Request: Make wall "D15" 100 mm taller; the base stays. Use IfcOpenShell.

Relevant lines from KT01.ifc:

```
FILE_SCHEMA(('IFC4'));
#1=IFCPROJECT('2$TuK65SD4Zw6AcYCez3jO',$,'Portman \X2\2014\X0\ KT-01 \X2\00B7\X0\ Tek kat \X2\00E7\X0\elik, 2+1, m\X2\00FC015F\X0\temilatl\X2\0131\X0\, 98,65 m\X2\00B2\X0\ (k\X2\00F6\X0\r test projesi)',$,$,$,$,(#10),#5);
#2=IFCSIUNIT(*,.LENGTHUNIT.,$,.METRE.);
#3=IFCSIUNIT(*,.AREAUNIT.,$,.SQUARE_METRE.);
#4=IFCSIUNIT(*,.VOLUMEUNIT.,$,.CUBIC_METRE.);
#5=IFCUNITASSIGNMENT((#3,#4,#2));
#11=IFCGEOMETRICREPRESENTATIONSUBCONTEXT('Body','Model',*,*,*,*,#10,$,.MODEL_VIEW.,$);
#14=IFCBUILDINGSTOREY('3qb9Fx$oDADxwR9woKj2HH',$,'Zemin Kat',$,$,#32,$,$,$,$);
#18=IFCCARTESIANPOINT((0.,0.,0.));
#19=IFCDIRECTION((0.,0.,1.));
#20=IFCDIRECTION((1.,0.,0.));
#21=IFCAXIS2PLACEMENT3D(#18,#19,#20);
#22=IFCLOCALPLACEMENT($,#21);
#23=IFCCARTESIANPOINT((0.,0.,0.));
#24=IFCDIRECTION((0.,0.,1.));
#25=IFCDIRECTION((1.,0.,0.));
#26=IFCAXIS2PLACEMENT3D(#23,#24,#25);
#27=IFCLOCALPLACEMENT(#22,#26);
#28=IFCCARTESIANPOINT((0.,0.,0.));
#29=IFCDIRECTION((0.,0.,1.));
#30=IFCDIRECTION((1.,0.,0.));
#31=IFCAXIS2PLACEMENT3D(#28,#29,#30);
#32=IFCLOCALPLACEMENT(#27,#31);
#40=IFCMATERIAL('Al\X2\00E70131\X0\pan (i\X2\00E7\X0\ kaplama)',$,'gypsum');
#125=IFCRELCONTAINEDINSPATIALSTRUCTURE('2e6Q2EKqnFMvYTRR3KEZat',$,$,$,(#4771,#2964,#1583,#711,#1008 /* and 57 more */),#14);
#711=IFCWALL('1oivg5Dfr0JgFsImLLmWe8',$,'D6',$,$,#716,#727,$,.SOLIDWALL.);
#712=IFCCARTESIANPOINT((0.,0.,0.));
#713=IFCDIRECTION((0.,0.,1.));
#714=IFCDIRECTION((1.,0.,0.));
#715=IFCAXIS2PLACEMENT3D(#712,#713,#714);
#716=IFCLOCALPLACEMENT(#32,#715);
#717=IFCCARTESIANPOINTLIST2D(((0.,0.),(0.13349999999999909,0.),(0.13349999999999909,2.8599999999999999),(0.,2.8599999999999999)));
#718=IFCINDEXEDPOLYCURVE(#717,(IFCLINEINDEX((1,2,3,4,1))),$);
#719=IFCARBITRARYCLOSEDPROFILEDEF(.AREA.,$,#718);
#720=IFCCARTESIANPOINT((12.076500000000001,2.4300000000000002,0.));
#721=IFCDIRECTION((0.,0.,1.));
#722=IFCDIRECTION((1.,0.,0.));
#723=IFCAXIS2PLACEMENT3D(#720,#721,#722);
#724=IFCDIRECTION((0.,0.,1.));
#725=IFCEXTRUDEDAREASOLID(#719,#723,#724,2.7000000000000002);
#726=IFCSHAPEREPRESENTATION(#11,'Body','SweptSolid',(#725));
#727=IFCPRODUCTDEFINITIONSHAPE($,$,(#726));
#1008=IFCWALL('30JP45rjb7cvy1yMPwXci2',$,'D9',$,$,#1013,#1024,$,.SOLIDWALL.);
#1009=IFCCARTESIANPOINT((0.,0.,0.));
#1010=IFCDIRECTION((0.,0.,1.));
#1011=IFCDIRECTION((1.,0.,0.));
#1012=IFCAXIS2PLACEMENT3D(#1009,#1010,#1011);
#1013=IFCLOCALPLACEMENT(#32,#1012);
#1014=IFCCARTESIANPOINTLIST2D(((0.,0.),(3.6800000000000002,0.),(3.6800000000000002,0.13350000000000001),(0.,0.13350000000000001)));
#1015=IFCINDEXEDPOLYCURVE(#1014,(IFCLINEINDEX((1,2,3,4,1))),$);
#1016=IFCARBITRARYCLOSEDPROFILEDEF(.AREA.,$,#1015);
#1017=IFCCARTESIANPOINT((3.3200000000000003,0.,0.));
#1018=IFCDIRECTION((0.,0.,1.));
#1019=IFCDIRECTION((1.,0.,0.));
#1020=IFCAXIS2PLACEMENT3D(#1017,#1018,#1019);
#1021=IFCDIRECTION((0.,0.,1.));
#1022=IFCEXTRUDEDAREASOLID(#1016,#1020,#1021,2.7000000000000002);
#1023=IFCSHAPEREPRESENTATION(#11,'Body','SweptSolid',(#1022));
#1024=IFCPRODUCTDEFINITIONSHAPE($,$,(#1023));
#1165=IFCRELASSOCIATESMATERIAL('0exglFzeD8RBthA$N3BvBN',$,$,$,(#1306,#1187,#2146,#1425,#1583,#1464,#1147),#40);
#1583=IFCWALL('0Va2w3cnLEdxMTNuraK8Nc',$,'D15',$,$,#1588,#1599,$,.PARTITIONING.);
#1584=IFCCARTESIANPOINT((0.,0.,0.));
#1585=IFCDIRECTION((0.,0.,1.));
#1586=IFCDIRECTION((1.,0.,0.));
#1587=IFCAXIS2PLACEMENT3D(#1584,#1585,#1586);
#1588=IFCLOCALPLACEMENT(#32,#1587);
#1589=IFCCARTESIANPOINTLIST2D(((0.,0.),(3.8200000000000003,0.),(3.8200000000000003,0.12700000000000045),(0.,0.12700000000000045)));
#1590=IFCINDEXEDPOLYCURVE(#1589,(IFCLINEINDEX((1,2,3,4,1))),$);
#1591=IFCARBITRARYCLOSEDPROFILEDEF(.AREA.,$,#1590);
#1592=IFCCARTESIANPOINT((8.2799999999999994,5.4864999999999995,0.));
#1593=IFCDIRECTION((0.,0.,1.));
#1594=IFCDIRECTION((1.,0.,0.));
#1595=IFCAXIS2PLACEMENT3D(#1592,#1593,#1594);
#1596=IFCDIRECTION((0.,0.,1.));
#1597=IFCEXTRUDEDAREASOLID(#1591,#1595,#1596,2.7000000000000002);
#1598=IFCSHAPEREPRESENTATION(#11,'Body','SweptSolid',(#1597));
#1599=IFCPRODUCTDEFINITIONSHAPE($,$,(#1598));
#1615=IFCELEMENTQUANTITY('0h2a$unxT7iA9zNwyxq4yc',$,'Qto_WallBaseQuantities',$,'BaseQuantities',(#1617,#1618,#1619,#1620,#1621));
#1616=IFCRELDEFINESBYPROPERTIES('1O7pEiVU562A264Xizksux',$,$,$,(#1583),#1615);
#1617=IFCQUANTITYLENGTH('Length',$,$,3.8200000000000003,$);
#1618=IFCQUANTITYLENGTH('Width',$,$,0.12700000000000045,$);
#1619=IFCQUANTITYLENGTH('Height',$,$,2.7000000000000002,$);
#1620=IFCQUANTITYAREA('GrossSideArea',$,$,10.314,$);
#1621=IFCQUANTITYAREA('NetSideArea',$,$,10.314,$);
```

```python
import ifcopenshell
import ifcopenshell.api.pset
import ifcopenshell.geom
import ifcopenshell.util.element
import ifcopenshell.util.representation
import ifcopenshell.util.shape
import ifcopenshell.util.unit

model = ifcopenshell.open("KT01.ifc")
unit_scale = ifcopenshell.util.unit.calculate_unit_scale(model)
area_scale = ifcopenshell.util.unit.calculate_unit_scale(model, "AREAUNIT")
settings = ifcopenshell.geom.settings()


def volume(element):
    """Net volume in cubic metres, openings subtracted."""
    shape = ifcopenshell.geom.create_shape(settings, element)
    return ifcopenshell.util.shape.get_volume(shape.geometry)


wall = model.by_guid("0Va2w3cnLEdxMTNuraK8Nc")
before = volume(wall)

body = ifcopenshell.util.representation.get_representation(wall, "Model", "Body")
solid = body.Items[0]
old_height = solid.Depth
solid.Depth += 0.1 / unit_scale
after = volume(wall)
thickness = 0.127  # wall thickness in metres

# Update the stored height, areas and volumes.
qto = model.by_id(ifcopenshell.util.element.get_pset(wall, "Qto_WallBaseQuantities", should_inherit=False)["id"])
ifcopenshell.api.pset.edit_qto(model, qto=qto, properties={
    "Height": solid.Depth,
    "GrossSideArea": ifcopenshell.util.element.get_pset(wall, "Qto_WallBaseQuantities", "GrossSideArea") * solid.Depth / old_height,
    "NetSideArea": after / thickness / area_scale,
})

print(f"height {old_height:g} -> {solid.Depth:g}, volume {before:.3f} -> {after:.3f} m3")

model.write("KT01_v2.ifc")
```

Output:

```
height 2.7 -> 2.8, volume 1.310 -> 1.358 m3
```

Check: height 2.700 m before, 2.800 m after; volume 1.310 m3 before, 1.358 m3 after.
